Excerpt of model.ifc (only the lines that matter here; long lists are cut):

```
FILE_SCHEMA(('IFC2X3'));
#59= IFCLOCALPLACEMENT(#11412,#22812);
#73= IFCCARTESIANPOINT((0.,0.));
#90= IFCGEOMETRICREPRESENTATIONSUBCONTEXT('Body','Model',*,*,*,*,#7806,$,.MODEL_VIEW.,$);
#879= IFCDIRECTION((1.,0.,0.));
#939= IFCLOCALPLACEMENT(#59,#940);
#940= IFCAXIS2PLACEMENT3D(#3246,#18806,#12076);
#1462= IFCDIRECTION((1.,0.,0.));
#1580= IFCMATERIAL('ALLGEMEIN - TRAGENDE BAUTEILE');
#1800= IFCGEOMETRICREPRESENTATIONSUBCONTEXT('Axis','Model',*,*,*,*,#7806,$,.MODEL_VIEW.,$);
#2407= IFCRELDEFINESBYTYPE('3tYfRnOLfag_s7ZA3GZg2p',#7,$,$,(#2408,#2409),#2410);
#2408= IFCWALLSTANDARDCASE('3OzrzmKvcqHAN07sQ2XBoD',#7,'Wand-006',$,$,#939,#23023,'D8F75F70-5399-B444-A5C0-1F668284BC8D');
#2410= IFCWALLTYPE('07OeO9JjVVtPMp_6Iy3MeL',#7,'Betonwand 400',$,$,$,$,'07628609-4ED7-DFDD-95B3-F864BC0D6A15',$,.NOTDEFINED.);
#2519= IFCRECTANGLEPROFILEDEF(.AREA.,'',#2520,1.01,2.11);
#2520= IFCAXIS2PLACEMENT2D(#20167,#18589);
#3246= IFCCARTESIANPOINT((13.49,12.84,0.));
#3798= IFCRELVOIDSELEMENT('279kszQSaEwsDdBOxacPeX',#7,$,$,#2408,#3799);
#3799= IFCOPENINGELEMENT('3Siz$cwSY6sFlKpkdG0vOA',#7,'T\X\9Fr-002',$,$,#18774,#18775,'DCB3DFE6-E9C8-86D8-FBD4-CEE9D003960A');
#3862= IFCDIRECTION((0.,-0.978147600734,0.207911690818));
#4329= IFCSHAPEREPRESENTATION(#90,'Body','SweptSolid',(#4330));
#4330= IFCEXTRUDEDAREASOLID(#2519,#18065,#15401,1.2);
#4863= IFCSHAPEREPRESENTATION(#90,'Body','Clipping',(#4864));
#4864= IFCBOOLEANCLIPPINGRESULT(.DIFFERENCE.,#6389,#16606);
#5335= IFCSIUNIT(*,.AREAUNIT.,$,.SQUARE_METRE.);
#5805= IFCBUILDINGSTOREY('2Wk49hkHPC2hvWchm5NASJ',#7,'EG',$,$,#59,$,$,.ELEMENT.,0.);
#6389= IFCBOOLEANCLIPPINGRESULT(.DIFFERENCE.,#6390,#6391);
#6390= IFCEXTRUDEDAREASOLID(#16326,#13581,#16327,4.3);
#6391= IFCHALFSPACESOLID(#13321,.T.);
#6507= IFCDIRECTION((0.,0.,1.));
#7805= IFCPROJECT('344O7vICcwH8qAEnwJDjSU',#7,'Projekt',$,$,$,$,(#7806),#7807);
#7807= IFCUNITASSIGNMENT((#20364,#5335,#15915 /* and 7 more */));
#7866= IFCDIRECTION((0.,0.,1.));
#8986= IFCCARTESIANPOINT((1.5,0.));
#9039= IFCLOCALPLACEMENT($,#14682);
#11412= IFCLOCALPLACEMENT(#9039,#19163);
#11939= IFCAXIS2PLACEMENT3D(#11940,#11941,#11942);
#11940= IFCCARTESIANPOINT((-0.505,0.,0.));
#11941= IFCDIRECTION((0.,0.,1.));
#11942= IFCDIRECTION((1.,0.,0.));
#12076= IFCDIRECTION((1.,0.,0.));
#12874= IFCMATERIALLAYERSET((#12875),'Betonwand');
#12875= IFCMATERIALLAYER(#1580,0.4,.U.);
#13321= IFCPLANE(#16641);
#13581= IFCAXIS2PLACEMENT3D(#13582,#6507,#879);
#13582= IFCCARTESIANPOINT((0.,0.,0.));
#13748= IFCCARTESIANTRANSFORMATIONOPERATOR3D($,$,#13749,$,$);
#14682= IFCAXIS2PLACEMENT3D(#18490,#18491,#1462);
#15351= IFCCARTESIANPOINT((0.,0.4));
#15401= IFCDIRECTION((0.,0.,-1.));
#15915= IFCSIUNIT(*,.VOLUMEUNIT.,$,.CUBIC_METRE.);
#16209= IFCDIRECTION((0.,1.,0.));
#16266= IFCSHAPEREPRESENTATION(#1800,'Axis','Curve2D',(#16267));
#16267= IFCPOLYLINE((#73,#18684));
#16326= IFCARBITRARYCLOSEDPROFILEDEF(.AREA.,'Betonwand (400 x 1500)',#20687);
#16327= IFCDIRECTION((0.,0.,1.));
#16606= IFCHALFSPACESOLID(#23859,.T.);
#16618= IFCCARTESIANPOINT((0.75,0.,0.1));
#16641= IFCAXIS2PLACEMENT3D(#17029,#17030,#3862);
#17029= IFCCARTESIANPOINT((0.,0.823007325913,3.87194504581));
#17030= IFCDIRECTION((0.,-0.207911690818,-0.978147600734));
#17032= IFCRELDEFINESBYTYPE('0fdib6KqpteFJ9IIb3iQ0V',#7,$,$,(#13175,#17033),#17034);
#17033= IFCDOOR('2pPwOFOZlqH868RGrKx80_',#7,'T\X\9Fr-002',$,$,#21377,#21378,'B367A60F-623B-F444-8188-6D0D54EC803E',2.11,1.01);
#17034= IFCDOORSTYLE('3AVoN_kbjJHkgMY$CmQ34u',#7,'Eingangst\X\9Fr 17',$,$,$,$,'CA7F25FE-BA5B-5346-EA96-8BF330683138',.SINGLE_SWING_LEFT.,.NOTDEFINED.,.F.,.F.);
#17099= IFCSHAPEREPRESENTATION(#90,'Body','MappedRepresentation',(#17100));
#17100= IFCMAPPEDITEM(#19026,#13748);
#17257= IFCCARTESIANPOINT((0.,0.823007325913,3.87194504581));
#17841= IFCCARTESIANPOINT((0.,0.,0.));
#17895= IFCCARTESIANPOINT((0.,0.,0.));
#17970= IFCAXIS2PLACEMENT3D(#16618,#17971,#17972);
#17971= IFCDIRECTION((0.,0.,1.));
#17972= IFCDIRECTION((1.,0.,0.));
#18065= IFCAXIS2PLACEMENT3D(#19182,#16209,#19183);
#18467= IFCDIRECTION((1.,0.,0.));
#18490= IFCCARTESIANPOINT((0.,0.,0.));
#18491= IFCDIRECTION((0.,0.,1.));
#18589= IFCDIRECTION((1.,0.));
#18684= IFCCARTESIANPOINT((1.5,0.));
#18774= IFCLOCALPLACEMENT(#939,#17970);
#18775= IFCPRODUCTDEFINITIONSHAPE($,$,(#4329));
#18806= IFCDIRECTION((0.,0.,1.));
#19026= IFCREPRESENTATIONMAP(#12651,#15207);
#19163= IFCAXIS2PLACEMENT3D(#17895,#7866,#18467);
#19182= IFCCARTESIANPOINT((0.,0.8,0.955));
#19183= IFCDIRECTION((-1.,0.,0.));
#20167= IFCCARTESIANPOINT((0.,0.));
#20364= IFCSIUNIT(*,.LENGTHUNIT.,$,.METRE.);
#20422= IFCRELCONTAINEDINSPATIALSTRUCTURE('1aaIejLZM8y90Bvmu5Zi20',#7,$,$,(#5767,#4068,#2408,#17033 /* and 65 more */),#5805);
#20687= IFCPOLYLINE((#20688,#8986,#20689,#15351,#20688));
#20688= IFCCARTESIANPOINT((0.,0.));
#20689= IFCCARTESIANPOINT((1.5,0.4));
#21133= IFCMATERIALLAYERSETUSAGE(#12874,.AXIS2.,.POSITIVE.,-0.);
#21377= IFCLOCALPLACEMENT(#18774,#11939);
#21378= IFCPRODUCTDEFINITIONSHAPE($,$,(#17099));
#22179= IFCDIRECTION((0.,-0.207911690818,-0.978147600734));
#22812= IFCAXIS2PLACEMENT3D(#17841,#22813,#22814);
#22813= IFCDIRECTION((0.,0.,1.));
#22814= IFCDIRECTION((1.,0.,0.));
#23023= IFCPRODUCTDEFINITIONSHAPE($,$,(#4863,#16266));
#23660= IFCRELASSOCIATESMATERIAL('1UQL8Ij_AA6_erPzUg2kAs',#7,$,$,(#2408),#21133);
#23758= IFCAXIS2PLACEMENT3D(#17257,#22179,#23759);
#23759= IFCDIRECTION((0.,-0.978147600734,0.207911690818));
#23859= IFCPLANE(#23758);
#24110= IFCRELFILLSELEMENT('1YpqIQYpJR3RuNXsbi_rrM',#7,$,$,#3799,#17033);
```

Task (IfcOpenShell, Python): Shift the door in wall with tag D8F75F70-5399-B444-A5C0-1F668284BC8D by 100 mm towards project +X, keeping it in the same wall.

```python
import ifcopenshell
import ifcopenshell.api.geometry
import ifcopenshell.util.placement

model = ifcopenshell.open("model.ifc")

door = model.by_guid("2pPwOFOZlqH868RGrKx80_")
opening = door.FillsVoids[0].RelatingOpeningElement
wall = opening.VoidsElements[0].RelatingBuildingElement

wall_matrix = ifcopenshell.util.placement.get_local_placement(wall.ObjectPlacement)
shift = wall_matrix[:3, 0] * 0.1
before = ifcopenshell.util.placement.get_local_placement(door.ObjectPlacement)[:3, 3].copy()

# The door is placed relative to its opening, so it follows when the opening moves.
matrix = ifcopenshell.util.placement.get_local_placement(opening.ObjectPlacement)
matrix[:3, 3] += shift
ifcopenshell.api.geometry.edit_object_placement(
    model, product=opening, matrix=matrix, is_si=False, should_transform_children=True
)

after = ifcopenshell.util.placement.get_local_placement(door.ObjectPlacement)[:3, 3]
print("door moved by", (after - before).round(3) + 0.0)

model.write("model_rev.ifc")
```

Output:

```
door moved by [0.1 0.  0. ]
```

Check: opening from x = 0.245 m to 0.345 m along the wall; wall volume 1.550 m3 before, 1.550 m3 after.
